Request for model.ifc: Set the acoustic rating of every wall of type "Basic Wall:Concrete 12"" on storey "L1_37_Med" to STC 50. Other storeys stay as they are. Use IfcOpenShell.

First a look at what the model holds.

```python
import ifcopenshell
import ifcopenshell.util.element

model = ifcopenshell.open("model.ifc")
print(model.schema)
storey = next(s for s in model.by_type("IfcBuildingStorey") if s.Name == "L1_37_Med")
walls = [e for e in ifcopenshell.util.element.get_decomposition(storey) if e.is_a("IfcWall")]
seen = {}
for e in walls:
    element_type = ifcopenshell.util.element.get_type(e)
    key = (element_type.Name if element_type != e and element_type else None, ifcopenshell.util.element.get_pset(e, "Pset_WallCommon", "AcousticRating"))
    seen[key] = seen.get(key, 0) + 1
for (name, value), count in sorted(seen.items(), key=str):
    print(count, "x", name, "|", value)
```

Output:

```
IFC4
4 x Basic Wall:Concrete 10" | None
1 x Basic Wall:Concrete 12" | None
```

```python
import ifcopenshell
import ifcopenshell.api.pset
import ifcopenshell.util.element

model = ifcopenshell.open("model.ifc")

storey = next(s for s in model.by_type("IfcBuildingStorey") if s.Name == "L1_37_Med")
walls = [e for e in ifcopenshell.util.element.get_decomposition(storey) if e.is_a("IfcWall")]

count = 0
for e in walls:
    element_type = ifcopenshell.util.element.get_type(e)
    if element_type in (None, e) or element_type.Name != 'Basic Wall:Concrete 12"':
        continue
    # add_pset returns the element's existing set when there is one.
    pset = ifcopenshell.api.pset.add_pset(model, product=e, name="Pset_WallCommon")
    ifcopenshell.api.pset.edit_pset(model, pset=pset, properties={"AcousticRating": "STC 50"})
    count += 1

print(count, "walls updated")

model.write("model_v2.ifc")
```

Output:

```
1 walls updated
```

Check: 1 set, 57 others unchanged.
